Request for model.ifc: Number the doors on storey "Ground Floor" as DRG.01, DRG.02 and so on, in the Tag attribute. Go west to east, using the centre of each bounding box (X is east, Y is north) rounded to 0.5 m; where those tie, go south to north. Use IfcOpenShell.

First a look at what the model holds.

```python
import ifcopenshell
import ifcopenshell.util.element
import ifcopenshell.util.placement

model = ifcopenshell.open("model.ifc")
print(model.schema)
storey = next(s for s in model.by_type("IfcBuildingStorey") if s.Name == "Ground Floor")
doors = [e for e in ifcopenshell.util.element.get_decomposition(storey) if e.is_a("IfcDoor")]
for e in sorted(doors, key=lambda e: e.id()):
    origin = ifcopenshell.util.placement.get_local_placement(e.ObjectPlacement)[:3, 3]
    print(e.id(), e.Tag, e.Name, origin.round(2) + 0.0, sep=" | ")
```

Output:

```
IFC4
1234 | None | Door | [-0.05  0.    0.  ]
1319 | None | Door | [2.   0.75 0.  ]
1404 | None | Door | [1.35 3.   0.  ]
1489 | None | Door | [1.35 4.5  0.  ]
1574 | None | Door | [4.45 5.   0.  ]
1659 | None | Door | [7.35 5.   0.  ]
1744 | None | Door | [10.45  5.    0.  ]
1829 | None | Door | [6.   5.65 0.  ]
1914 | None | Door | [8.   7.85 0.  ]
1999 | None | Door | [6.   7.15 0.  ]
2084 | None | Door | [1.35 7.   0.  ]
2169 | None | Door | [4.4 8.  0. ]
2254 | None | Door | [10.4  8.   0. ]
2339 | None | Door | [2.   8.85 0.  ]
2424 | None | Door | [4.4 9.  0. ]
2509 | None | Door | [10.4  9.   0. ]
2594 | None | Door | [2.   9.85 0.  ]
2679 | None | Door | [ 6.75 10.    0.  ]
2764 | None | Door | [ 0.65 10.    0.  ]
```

```python
import ifcopenshell
import ifcopenshell.geom
import ifcopenshell.util.element
import ifcopenshell.util.shape

model = ifcopenshell.open("model.ifc")
settings = ifcopenshell.geom.settings()
settings.set("use-world-coords", True)


def centre(element):
    shape = ifcopenshell.geom.create_shape(settings, element)
    return ifcopenshell.util.shape.get_bbox_centroid(shape.geometry)


storey = next(s for s in model.by_type("IfcBuildingStorey") if s.Name == "Ground Floor")
doors = [e for e in ifcopenshell.util.element.get_decomposition(storey) if e.is_a("IfcDoor")]

# Insertion points can sit at a corner or the storey origin, so sort by the geometry (in metres).
centres = {e: centre(e) for e in doors}
doors.sort(key=lambda e: (round(centres[e][0] / 0.5), centres[e][1]))

for i, e in enumerate(doors, start=1):
    number = f"DRG.{i:02d}"
    e.Tag = number
    print(e.id(), number)

model.write("model_v2.ifc")
```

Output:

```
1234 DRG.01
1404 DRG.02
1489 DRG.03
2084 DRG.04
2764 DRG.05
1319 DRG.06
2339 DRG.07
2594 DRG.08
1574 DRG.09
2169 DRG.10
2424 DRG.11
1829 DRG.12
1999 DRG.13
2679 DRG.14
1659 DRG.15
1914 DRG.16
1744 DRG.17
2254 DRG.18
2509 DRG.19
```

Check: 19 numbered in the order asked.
